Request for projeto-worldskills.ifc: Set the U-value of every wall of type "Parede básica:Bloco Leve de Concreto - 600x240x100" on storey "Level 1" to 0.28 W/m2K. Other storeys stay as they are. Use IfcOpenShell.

First a look at what the model holds.

```python
import ifcopenshell
import ifcopenshell.util.element

model = ifcopenshell.open("projeto-worldskills.ifc")
print(model.schema)
storey = next(s for s in model.by_type("IfcBuildingStorey") if s.Name == "Level 1")
walls = [e for e in ifcopenshell.util.element.get_decomposition(storey) if e.is_a("IfcWall")]
seen = {}
for e in walls:
    element_type = ifcopenshell.util.element.get_type(e)
    key = (element_type.Name if element_type != e and element_type else None, ifcopenshell.util.element.get_pset(e, "Pset_WallCommon", "ThermalTransmittance"))
    seen[key] = seen.get(key, 0) + 1
for (name, value), count in sorted(seen.items(), key=str):
    print(count, "x", name, "|", value)
```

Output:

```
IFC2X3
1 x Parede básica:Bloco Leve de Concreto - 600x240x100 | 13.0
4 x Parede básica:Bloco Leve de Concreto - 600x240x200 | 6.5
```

```python
import ifcopenshell
import ifcopenshell.api.pset
import ifcopenshell.util.element

model = ifcopenshell.open("projeto-worldskills.ifc")

storey = next(s for s in model.by_type("IfcBuildingStorey") if s.Name == "Level 1")
walls = [e for e in ifcopenshell.util.element.get_decomposition(storey) if e.is_a("IfcWall")]

count = 0
for e in walls:
    element_type = ifcopenshell.util.element.get_type(e)
    if element_type in (None, e) or element_type.Name != "Parede básica:Bloco Leve de Concreto - 600x240x100":
        continue
    # add_pset returns the element's existing set when there is one.
    pset = ifcopenshell.api.pset.add_pset(model, product=e, name="Pset_WallCommon")
    ifcopenshell.api.pset.edit_pset(model, pset=pset, properties={"ThermalTransmittance": 0.28})
    count += 1

print(count, "walls updated")

model.write("projeto-worldskills-out.ifc")
```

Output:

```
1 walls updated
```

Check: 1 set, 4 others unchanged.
